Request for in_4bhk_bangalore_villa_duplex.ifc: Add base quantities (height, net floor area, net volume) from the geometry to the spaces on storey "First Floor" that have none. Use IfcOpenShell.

First a look at what the model holds.

```python
import ifcopenshell
import ifcopenshell.util.element
import ifcopenshell.util.unit

model = ifcopenshell.open("in_4bhk_bangalore_villa_duplex.ifc")
print(model.schema)
for unit_type in ("LENGTHUNIT", "AREAUNIT", "VOLUMEUNIT"):
    print(unit_type, ifcopenshell.util.unit.calculate_unit_scale(model, unit_type))
storey = next(s for s in model.by_type("IfcBuildingStorey") if s.Name == "First Floor")
spaces = [e for e in ifcopenshell.util.element.get_decomposition(storey) if e.is_a("IfcSpace")]
for e in sorted(spaces, key=lambda e: e.id()):
    print(e.id(), e.is_a(), e.Name, list(ifcopenshell.util.element.get_psets(e, qtos_only=True)), sep=" | ")
```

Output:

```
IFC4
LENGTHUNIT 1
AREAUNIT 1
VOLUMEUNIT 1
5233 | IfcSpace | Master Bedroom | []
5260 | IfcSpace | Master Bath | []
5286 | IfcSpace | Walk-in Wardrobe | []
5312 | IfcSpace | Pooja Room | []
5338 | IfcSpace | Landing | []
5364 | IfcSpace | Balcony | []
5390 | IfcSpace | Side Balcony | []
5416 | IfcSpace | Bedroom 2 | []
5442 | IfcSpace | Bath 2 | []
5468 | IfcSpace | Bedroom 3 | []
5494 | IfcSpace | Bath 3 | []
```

```python
import ifcopenshell
import ifcopenshell.api.pset
import ifcopenshell.geom
import ifcopenshell.util.element
import ifcopenshell.util.shape
import ifcopenshell.util.unit

model = ifcopenshell.open("in_4bhk_bangalore_villa_duplex.ifc")
unit_scale = ifcopenshell.util.unit.calculate_unit_scale(model)
area_scale = ifcopenshell.util.unit.calculate_unit_scale(model, "AREAUNIT")
volume_scale = ifcopenshell.util.unit.calculate_unit_scale(model, "VOLUMEUNIT")
settings = ifcopenshell.geom.settings()

storey = next(s for s in model.by_type("IfcBuildingStorey") if s.Name == "First Floor")
spaces = [e for e in ifcopenshell.util.element.get_decomposition(storey) if e.is_a("IfcSpace")]

for e in sorted(spaces, key=lambda e: e.id()):
    if ifcopenshell.util.element.get_psets(e, qtos_only=True, should_inherit=False):
        continue
    # Geometry comes back in metres, in the element's own axes.
    shape = ifcopenshell.geom.create_shape(settings, e)
    values = {
        "Height": ifcopenshell.util.shape.get_z(shape.geometry) / unit_scale,
        "NetFloorArea": ifcopenshell.util.shape.get_footprint_area(shape.geometry) / area_scale,
        "NetVolume": ifcopenshell.util.shape.get_volume(shape.geometry) / volume_scale,
    }
    qto = ifcopenshell.api.pset.add_qto(model, product=e, name="Qto_SpaceBaseQuantities")
    ifcopenshell.api.pset.edit_qto(model, qto=qto, properties=values)
    print(e.id(), {k: round(v, 3) for k, v in values.items()})

model.write("in_4bhk_bangalore_villa_duplex-out.ifc")
```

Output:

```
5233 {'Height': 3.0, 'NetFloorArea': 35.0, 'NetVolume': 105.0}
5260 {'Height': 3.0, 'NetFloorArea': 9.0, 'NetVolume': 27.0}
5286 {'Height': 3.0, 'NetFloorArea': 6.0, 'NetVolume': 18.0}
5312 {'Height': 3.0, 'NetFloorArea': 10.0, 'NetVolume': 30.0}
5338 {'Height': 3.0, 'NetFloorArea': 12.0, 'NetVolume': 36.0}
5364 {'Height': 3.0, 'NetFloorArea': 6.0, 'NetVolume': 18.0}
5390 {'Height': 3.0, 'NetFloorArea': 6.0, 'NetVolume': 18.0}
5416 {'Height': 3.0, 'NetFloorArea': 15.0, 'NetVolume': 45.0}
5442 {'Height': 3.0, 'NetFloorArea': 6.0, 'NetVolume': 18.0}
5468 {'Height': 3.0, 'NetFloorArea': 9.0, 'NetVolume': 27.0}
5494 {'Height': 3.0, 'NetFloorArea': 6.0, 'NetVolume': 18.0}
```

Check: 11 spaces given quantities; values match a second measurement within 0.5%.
